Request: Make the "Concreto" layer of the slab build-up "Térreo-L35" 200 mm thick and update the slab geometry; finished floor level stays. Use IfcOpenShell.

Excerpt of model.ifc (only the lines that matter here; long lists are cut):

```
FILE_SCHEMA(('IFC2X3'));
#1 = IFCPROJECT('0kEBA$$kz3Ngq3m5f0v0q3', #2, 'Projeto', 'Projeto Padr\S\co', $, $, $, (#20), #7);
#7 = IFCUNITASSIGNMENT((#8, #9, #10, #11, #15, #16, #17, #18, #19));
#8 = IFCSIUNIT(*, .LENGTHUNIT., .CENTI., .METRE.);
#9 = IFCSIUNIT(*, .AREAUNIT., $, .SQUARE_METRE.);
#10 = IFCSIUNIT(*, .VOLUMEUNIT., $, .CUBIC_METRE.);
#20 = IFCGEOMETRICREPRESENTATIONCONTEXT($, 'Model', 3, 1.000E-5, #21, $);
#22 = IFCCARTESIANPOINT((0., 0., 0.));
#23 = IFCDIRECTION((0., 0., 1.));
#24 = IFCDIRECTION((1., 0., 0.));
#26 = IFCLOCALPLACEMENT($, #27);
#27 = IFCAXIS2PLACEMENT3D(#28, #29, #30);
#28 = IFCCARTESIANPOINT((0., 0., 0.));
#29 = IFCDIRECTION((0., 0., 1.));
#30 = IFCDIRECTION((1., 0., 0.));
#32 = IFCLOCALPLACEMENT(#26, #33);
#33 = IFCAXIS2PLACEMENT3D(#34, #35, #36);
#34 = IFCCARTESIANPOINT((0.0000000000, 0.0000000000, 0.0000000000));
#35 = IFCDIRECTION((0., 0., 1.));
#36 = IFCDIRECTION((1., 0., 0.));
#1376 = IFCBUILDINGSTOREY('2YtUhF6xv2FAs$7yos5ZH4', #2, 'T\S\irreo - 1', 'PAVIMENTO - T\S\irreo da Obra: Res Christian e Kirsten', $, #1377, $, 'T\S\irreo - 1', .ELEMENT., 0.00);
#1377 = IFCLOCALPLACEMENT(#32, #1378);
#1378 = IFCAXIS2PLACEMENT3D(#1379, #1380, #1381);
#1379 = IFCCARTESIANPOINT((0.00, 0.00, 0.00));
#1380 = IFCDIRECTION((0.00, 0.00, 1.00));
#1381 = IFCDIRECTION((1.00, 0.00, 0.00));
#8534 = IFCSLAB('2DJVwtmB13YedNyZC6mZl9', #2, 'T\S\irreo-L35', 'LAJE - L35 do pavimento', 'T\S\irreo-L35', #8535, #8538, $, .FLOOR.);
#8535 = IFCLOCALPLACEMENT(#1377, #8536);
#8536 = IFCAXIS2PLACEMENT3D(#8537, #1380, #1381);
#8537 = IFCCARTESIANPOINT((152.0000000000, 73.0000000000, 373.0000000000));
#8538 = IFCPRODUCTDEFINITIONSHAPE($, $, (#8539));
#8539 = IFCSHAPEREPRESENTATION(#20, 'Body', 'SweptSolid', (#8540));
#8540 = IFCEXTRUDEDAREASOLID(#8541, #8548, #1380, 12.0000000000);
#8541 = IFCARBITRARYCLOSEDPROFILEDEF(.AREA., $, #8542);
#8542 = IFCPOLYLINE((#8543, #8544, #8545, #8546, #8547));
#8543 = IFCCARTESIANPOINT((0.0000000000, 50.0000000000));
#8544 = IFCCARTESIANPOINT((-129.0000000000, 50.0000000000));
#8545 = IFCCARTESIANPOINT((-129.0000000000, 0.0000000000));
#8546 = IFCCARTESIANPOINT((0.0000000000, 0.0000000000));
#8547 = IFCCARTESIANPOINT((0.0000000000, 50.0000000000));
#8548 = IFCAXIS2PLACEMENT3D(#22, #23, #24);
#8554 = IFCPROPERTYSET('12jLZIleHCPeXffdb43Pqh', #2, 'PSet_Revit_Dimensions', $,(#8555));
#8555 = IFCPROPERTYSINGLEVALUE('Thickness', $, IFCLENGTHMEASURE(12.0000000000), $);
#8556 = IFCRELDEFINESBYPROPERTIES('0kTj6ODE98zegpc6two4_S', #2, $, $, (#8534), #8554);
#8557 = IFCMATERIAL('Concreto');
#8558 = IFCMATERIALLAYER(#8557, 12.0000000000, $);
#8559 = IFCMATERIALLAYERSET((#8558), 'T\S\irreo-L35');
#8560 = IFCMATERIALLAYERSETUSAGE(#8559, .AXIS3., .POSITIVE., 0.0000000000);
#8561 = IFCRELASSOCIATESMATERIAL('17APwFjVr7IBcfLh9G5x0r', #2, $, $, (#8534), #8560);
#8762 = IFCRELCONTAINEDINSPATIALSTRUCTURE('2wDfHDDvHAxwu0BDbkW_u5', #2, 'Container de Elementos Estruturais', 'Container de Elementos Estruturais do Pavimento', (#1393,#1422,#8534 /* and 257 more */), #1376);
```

```python
import ifcopenshell
import ifcopenshell.api.pset
import ifcopenshell.util.element
import ifcopenshell.util.unit

model = ifcopenshell.open("model.ifc")
unit_scale = ifcopenshell.util.unit.calculate_unit_scale(model)

layer_set = model.by_id(8559)
layer = next(l for l in layer_set.MaterialLayers if l.Material and l.Material.Name == "Concreto")
change = 0.2 / unit_scale - layer.LayerThickness
layer.LayerThickness += change

# Geometry does not follow the layer set by itself.
slabs = [e for e in ifcopenshell.util.element.get_elements_by_material(model, layer_set) if e.is_a("IfcSlab")]
for slab in sorted(slabs, key=lambda e: e.id()):
    body = next(r for r in slab.Representation.Representations if r.RepresentationIdentifier == "Body")
    solid = body.Items[0]
    old_depth = solid.Depth
    solid.Depth += change
    # Extruded upwards: lower the start of the extrusion so the top stays.
    x, y, z = solid.Position.Location.Coordinates
    solid.Position.Location = model.createIfcCartesianPoint((x, y, z - change))
    pset = model.by_id(ifcopenshell.util.element.get_pset(slab, "PSet_Revit_Dimensions", should_inherit=False)["id"])
    ifcopenshell.api.pset.edit_pset(model, pset=pset, properties={
        "Thickness": model.create_entity("IfcLengthMeasure", solid.Depth),
    })
    print(slab.id(), f"{old_depth:g} -> {solid.Depth:g}")

# The layers are counted up from the underside, which has moved.
for usage in {ifcopenshell.util.element.get_material(slab) for slab in slabs}:
    usage.OffsetFromReferenceLine -= change

model.write("model_rev.ifc")
```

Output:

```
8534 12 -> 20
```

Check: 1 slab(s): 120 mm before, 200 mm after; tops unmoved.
